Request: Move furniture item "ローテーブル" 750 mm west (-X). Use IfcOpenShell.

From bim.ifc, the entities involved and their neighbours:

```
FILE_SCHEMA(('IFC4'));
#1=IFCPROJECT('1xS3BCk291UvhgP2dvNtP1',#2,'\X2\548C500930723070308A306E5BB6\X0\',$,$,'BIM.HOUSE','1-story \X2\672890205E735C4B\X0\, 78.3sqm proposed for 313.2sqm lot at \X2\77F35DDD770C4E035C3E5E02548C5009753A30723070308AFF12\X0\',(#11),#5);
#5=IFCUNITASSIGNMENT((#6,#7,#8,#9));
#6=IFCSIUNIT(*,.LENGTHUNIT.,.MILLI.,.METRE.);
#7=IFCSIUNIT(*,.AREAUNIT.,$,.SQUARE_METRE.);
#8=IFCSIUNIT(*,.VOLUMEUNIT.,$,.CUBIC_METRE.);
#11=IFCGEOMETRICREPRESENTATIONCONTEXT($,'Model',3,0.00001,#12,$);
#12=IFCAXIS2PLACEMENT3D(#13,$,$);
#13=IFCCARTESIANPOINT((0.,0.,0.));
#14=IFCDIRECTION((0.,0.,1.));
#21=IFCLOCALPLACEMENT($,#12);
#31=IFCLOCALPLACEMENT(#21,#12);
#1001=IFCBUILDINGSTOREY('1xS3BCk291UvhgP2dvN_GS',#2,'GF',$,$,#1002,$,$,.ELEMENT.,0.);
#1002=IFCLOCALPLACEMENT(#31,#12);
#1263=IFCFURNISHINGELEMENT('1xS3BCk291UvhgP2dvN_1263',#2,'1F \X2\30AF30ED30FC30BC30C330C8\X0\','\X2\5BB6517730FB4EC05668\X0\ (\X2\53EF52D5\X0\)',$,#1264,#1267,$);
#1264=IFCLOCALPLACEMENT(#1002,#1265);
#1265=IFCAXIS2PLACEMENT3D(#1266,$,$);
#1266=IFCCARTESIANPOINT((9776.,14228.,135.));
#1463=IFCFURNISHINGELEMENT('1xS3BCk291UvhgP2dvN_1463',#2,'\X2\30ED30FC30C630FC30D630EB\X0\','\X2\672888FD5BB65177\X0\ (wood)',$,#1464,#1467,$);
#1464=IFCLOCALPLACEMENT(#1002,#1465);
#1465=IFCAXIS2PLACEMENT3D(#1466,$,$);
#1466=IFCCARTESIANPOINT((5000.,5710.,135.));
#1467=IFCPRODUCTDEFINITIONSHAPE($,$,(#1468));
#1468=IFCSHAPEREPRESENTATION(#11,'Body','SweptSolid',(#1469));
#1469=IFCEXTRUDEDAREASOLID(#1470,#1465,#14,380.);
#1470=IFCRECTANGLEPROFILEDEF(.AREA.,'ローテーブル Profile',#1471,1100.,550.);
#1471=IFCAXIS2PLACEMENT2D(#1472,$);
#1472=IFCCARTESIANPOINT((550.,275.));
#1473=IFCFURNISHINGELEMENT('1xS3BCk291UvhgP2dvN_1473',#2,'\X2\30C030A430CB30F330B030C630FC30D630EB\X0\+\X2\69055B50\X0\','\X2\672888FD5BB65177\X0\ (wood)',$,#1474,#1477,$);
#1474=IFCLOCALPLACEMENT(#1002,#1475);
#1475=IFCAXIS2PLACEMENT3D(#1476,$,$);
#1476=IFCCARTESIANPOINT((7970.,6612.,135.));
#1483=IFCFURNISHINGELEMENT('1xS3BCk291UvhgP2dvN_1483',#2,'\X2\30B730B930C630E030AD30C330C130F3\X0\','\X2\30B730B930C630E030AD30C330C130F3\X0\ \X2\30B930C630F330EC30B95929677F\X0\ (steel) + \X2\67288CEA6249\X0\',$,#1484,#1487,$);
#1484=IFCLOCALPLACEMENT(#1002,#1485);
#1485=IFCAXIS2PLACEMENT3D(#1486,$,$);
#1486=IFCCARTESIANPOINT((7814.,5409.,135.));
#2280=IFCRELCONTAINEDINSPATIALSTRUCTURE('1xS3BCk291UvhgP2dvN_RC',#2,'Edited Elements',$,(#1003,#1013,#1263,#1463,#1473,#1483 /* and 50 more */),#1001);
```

```python
import ifcopenshell
import ifcopenshell.api.geometry
import ifcopenshell.util.placement
import ifcopenshell.util.unit

model = ifcopenshell.open("bim.ifc")
unit_scale = ifcopenshell.util.unit.calculate_unit_scale(model)

item = model.by_id(1463)
matrix = ifcopenshell.util.placement.get_local_placement(item.ObjectPlacement)
matrix[0, 3] -= 0.75 / unit_scale
ifcopenshell.api.geometry.edit_object_placement(model, product=item, matrix=matrix, is_si=False)

print(ifcopenshell.util.placement.get_local_placement(item.ObjectPlacement).round(3) + 0.0)

model.write("bim-out.ifc")
```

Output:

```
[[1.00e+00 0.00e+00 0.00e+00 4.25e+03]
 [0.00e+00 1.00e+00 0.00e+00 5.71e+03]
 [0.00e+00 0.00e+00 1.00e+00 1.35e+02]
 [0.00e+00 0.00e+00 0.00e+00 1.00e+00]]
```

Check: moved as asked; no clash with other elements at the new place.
